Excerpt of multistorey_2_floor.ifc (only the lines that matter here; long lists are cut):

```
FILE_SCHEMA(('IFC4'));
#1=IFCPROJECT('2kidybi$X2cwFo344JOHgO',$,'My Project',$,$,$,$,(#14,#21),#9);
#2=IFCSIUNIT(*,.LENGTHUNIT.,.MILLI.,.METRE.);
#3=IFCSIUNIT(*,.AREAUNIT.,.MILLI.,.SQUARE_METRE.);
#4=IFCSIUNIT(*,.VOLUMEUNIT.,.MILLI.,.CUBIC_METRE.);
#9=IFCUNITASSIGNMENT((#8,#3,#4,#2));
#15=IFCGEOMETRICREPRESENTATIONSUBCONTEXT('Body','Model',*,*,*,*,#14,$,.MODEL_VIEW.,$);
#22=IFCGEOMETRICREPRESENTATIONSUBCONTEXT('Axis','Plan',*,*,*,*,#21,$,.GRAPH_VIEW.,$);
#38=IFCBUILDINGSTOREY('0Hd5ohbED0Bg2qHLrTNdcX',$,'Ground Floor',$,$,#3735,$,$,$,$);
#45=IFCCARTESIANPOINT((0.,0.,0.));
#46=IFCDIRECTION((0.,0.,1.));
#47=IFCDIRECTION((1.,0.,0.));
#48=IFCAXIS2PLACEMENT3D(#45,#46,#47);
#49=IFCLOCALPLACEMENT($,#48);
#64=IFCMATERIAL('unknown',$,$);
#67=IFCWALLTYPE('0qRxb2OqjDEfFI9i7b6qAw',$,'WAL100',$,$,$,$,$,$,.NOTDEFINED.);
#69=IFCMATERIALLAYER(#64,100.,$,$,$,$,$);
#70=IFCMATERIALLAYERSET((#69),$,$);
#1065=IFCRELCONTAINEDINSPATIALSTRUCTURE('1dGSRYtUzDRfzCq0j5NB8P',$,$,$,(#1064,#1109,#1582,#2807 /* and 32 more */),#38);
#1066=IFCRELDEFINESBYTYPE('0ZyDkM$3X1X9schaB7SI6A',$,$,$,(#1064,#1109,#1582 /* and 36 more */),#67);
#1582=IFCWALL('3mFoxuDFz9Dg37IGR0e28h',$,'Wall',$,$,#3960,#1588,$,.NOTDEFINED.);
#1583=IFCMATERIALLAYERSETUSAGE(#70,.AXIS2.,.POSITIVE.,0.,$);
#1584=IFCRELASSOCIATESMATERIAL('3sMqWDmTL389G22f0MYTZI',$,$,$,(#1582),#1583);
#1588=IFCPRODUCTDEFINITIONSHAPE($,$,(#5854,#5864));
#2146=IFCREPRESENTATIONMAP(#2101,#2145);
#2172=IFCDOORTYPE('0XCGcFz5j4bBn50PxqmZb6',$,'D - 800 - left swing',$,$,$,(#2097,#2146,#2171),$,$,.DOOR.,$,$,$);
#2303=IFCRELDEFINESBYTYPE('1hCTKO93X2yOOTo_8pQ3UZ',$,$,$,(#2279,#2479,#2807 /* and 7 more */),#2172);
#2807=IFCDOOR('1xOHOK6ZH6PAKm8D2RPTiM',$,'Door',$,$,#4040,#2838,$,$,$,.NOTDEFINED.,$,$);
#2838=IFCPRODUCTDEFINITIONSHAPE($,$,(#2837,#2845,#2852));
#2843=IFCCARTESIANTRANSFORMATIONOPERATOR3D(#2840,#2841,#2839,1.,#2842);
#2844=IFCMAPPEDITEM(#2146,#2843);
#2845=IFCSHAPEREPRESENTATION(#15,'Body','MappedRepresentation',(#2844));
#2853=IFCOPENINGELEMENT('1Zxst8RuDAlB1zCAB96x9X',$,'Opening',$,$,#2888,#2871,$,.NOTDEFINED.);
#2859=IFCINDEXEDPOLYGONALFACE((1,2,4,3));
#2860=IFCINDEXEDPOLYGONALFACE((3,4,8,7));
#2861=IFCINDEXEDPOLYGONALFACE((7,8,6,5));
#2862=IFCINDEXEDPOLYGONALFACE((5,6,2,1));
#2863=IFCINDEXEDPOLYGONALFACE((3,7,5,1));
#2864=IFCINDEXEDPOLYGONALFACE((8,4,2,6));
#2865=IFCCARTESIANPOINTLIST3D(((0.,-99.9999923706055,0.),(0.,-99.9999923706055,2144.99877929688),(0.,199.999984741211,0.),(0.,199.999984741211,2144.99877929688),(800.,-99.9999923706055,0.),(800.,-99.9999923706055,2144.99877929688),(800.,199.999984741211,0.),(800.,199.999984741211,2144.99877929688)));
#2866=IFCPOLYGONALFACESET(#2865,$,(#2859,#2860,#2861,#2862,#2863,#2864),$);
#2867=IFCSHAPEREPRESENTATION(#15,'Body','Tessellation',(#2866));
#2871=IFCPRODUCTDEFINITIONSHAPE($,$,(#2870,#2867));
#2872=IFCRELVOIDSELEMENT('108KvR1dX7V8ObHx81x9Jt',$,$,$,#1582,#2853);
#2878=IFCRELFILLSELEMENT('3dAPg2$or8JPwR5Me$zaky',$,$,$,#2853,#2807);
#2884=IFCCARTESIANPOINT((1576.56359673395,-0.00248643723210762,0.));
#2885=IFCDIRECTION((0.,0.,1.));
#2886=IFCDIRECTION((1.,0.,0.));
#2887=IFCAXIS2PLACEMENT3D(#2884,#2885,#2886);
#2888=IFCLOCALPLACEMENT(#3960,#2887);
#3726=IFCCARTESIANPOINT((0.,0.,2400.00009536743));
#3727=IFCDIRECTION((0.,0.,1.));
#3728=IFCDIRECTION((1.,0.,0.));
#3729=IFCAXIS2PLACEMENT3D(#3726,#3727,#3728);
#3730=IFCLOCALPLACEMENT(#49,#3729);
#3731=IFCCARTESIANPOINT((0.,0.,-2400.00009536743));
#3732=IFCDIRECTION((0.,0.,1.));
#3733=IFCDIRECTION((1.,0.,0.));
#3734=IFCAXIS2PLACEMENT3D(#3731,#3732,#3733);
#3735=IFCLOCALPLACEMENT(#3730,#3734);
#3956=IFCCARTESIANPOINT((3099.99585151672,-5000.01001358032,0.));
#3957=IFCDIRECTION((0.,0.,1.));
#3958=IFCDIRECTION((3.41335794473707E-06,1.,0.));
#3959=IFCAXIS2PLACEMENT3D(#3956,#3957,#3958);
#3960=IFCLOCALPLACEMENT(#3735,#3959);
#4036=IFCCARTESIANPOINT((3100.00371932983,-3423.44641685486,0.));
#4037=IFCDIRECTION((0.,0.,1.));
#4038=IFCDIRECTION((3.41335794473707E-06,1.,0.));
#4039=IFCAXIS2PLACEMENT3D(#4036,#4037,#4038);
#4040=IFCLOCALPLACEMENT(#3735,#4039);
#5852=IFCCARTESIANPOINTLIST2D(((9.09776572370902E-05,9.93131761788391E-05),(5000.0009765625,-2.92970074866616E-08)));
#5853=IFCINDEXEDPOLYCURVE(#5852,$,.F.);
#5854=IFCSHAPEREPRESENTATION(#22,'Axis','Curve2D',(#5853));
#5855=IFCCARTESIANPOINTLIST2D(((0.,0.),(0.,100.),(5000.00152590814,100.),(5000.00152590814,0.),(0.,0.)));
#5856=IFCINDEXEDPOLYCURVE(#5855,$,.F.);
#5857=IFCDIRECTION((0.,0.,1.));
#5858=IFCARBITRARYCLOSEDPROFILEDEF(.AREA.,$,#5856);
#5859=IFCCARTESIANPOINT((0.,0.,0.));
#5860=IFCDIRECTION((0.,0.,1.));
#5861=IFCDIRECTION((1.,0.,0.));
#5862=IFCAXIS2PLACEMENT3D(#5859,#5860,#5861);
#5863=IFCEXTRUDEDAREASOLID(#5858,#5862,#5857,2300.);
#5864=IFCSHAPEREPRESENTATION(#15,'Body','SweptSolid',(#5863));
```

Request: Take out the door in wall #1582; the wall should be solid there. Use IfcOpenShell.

```python
import ifcopenshell
import ifcopenshell.api.feature
import ifcopenshell.api.root
import ifcopenshell.geom
import ifcopenshell.util.shape

model = ifcopenshell.open("multistorey_2_floor.ifc")
settings = ifcopenshell.geom.settings()


def volume(element):
    """Net volume in cubic metres, openings subtracted."""
    shape = ifcopenshell.geom.create_shape(settings, element)
    return ifcopenshell.util.shape.get_volume(shape.geometry)


door = model.by_guid("1xOHOK6ZH6PAKm8D2RPTiM")
opening = door.FillsVoids[0].RelatingOpeningElement
wall = opening.VoidsElements[0].RelatingBuildingElement
before = volume(wall)

ifcopenshell.api.root.remove_product(model, product=door)
ifcopenshell.api.feature.remove_feature(model, feature=opening)

after = volume(wall)

print(f"wall volume {before:.3f} -> {after:.3f} m3")

model.write("multistorey_2_floor_edited.ifc")
```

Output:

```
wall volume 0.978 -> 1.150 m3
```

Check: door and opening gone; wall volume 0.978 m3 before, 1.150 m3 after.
